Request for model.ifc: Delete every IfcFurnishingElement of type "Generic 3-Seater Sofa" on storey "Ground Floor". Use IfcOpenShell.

First a look at what the model holds.

```python
import ifcopenshell
import ifcopenshell.util.element

model = ifcopenshell.open("model.ifc")
print(model.schema)
storey = next(s for s in model.by_type("IfcBuildingStorey") if s.Name == "Ground Floor")
furniture = [e for e in ifcopenshell.util.element.get_decomposition(storey) if e.is_a("IfcFurnishingElement")]
seen = {}
for e in furniture:
    element_type = ifcopenshell.util.element.get_type(e)
    name = element_type.Name if element_type not in (None, e) else None
    seen[name] = seen.get(name, 0) + 1
for name, count in sorted(seen.items(), key=str):
    print(count, "x", name)
```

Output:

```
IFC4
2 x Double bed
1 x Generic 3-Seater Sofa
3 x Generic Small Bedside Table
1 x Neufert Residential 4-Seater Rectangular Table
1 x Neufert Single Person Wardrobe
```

```python
import ifcopenshell
import ifcopenshell.api.root
import ifcopenshell.util.element

model = ifcopenshell.open("model.ifc")

storey = next(s for s in model.by_type("IfcBuildingStorey") if s.Name == "Ground Floor")
furniture = [e for e in ifcopenshell.util.element.get_decomposition(storey) if e.is_a("IfcFurnishingElement")]
targets = [e for e in furniture if (t := ifcopenshell.util.element.get_type(e)) not in (None, e) and t.Name == "Generic 3-Seater Sofa"]

for e in targets:
    ifcopenshell.api.root.remove_product(model, product=e)
print(len(targets), "removed")

model.write("model_rev.ifc")
```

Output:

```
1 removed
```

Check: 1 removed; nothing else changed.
